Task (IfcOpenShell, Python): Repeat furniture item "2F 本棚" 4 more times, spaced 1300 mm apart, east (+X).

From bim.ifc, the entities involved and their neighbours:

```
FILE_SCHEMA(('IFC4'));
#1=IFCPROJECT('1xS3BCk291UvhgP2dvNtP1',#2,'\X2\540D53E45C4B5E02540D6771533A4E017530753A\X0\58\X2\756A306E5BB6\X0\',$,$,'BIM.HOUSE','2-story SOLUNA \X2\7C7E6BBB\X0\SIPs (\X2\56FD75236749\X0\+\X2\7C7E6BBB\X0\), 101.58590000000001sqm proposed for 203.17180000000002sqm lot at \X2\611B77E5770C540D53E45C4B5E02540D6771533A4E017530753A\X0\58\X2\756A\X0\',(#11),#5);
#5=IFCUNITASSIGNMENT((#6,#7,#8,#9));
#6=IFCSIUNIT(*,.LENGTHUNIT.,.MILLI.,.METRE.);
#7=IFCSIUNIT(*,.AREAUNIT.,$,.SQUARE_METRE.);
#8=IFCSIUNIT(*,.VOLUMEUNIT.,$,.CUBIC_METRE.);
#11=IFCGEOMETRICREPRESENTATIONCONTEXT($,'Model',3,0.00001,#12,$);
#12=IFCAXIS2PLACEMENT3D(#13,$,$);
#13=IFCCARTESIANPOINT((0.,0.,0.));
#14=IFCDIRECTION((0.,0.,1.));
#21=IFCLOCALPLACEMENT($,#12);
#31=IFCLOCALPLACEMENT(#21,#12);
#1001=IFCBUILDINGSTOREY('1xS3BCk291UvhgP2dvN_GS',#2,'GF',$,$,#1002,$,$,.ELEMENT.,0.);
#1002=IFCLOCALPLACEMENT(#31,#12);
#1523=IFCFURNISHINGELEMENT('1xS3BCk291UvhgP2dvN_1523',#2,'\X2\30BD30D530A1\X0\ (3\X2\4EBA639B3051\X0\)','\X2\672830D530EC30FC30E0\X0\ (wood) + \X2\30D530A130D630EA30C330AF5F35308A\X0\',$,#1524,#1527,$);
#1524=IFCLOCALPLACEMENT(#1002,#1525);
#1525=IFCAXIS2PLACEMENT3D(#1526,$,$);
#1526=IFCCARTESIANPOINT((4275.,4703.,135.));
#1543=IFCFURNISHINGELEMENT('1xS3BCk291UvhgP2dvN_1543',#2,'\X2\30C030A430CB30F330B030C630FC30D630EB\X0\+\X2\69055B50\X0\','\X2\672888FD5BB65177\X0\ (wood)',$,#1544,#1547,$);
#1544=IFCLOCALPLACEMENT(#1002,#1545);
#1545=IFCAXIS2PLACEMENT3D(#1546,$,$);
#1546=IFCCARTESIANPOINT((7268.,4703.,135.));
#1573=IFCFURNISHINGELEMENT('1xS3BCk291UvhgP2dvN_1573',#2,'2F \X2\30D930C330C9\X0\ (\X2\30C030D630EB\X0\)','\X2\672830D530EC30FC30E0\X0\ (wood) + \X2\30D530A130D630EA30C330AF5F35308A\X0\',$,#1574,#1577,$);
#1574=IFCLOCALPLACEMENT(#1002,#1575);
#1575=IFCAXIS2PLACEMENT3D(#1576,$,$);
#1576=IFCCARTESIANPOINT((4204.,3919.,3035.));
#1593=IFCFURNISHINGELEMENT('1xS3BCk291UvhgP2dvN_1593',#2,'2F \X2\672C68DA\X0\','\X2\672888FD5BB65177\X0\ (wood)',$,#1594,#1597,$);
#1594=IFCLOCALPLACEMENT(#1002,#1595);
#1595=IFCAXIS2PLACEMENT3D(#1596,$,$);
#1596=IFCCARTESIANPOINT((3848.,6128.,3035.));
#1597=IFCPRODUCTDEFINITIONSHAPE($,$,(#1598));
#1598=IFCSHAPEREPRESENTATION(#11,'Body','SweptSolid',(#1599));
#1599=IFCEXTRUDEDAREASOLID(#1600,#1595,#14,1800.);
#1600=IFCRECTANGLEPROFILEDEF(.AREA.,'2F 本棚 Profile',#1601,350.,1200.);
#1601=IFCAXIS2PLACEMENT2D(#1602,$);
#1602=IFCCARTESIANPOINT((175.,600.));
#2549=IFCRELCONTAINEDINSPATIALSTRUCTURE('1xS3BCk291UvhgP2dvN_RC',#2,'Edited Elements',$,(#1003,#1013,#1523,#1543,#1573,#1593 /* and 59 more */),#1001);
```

```python
import numpy as np
import ifcopenshell
import ifcopenshell.api.geometry
import ifcopenshell.api.root
import ifcopenshell.util.element
import ifcopenshell.util.placement
import ifcopenshell.util.unit

model = ifcopenshell.open("bim.ifc")
unit_scale = ifcopenshell.util.unit.calculate_unit_scale(model)


def reuse_history(source, copy):
    """copy_class also copies each property set's owner history, people and application; keep the originals."""
    for rel in copy.IsDefinedBy:
        if rel.is_a("IfcRelDefinesByProperties") and (history := rel.RelatingPropertyDefinition.OwnerHistory):
            rel.RelatingPropertyDefinition.OwnerHistory = source.OwnerHistory
            ifcopenshell.util.element.remove_deep2(model, history)


source = model.by_guid("1xS3BCk291UvhgP2dvN_1593")
base = ifcopenshell.util.placement.get_local_placement(source.ObjectPlacement)
step = np.array([1.0, 0.0, 0.0]) * 1.3 / unit_scale

for i in range(1, 5):
    copy = ifcopenshell.api.root.copy_class(model, product=source)
    copy.Representation = ifcopenshell.util.element.copy_deep(
        model, source.Representation, exclude=["IfcGeometricRepresentationContext", "IfcRepresentationMap"]
    )
    reuse_history(source, copy)
    matrix = base.copy()
    matrix[:3, 3] += i * step
    print("added at", matrix[:3, 3].round(3) + 0.0)
    ifcopenshell.api.geometry.edit_object_placement(model, product=copy, matrix=matrix, is_si=False)

model.write("bim_updated.ifc")
```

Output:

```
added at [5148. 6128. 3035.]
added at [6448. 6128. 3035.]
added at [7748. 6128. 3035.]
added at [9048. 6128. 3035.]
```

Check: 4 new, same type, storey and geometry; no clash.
